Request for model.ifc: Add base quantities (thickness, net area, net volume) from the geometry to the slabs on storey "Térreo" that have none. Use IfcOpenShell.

First a look at what the model holds.

```python
import ifcopenshell
import ifcopenshell.util.element
import ifcopenshell.util.unit

model = ifcopenshell.open("model.ifc")
print(model.schema)
for unit_type in ("LENGTHUNIT", "AREAUNIT", "VOLUMEUNIT"):
    print(unit_type, ifcopenshell.util.unit.calculate_unit_scale(model, unit_type))
storey = next(s for s in model.by_type("IfcBuildingStorey") if s.Name == "Térreo")
slabs = [e for e in ifcopenshell.util.element.get_decomposition(storey) if e.is_a("IfcSlab")]
for e in sorted(slabs, key=lambda e: e.id()):
    print(e.id(), e.is_a(), e.Name, list(ifcopenshell.util.element.get_psets(e, qtos_only=True)), sep=" | ")
```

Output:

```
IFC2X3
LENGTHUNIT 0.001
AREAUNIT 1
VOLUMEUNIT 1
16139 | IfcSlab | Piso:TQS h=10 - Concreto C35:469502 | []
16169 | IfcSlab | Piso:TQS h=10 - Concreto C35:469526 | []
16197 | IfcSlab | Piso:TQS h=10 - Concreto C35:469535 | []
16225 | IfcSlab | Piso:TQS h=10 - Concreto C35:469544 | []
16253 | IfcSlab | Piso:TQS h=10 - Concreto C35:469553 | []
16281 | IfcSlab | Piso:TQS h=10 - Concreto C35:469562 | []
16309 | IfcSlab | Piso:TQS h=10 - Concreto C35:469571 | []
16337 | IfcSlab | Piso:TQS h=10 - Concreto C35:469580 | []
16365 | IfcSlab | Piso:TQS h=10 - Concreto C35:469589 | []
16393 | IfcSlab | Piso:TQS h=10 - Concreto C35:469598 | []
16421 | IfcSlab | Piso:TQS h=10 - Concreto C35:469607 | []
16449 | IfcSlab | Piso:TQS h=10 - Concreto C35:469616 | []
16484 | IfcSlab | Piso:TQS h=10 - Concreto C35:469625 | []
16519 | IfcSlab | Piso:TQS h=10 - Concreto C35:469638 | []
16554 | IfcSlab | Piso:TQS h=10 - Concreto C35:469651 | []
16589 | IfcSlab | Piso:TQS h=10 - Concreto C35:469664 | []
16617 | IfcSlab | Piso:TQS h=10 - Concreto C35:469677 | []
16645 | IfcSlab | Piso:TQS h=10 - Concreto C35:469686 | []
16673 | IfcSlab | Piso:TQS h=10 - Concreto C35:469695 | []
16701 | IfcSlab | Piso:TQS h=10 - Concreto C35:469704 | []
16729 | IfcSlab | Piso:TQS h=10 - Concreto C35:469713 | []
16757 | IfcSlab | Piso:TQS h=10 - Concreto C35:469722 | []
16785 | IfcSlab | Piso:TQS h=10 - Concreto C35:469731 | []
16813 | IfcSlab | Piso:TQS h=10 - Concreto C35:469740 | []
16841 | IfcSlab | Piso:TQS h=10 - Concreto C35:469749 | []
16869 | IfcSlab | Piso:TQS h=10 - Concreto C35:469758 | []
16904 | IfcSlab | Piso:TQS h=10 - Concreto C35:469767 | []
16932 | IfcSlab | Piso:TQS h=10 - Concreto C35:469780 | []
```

```python
import ifcopenshell
import ifcopenshell.api.pset
import ifcopenshell.geom
import ifcopenshell.util.element
import ifcopenshell.util.shape
import ifcopenshell.util.unit

model = ifcopenshell.open("model.ifc")
unit_scale = ifcopenshell.util.unit.calculate_unit_scale(model)
area_scale = ifcopenshell.util.unit.calculate_unit_scale(model, "AREAUNIT")
volume_scale = ifcopenshell.util.unit.calculate_unit_scale(model, "VOLUMEUNIT")
settings = ifcopenshell.geom.settings()

storey = next(s for s in model.by_type("IfcBuildingStorey") if s.Name == "Térreo")
slabs = [e for e in ifcopenshell.util.element.get_decomposition(storey) if e.is_a("IfcSlab")]

for e in sorted(slabs, key=lambda e: e.id()):
    if ifcopenshell.util.element.get_psets(e, qtos_only=True, should_inherit=False):
        continue
    # Geometry comes back in metres, in the element's own axes.
    shape = ifcopenshell.geom.create_shape(settings, e)
    values = {
        "Width": ifcopenshell.util.shape.get_z(shape.geometry) / unit_scale,
        "NetArea": ifcopenshell.util.shape.get_footprint_area(shape.geometry) / area_scale,
        "NetVolume": ifcopenshell.util.shape.get_volume(shape.geometry) / volume_scale,
    }
    qto = ifcopenshell.api.pset.add_qto(model, product=e, name="BaseQuantities")
    ifcopenshell.api.pset.edit_qto(model, qto=qto, properties=values)
    print(e.id(), {k: round(v, 3) for k, v in values.items()})

model.write("model_edited.ifc")
```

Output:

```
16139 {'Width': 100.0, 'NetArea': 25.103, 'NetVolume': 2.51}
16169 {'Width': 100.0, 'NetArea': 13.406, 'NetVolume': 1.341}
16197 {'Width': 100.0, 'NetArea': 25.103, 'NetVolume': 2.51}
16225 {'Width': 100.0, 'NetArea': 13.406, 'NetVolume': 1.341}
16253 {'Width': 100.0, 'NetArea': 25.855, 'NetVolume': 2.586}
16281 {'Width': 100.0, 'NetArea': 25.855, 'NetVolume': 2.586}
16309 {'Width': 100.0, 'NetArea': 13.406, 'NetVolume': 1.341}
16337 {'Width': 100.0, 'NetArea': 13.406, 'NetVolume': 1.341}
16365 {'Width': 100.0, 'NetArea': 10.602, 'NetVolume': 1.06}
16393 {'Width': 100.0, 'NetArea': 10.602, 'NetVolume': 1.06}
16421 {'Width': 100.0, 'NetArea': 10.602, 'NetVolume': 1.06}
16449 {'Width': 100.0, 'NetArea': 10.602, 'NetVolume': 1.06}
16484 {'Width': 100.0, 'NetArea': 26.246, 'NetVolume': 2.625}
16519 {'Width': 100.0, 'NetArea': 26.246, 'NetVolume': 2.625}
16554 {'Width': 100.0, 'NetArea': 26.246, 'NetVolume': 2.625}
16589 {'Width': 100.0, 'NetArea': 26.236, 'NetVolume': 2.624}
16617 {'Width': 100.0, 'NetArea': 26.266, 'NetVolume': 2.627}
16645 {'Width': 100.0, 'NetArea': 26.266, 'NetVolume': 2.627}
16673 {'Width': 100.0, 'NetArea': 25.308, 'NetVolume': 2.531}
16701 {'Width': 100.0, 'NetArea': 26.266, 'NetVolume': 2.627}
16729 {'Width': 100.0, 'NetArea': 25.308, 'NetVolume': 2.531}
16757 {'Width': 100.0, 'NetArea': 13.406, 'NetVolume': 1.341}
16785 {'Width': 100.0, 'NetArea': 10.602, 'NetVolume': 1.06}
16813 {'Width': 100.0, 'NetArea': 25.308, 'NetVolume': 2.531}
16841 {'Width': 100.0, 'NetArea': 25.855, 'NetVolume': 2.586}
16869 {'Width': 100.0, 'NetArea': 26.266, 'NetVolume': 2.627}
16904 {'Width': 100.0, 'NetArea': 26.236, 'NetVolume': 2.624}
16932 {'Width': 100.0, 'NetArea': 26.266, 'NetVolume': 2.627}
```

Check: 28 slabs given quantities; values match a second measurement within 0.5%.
